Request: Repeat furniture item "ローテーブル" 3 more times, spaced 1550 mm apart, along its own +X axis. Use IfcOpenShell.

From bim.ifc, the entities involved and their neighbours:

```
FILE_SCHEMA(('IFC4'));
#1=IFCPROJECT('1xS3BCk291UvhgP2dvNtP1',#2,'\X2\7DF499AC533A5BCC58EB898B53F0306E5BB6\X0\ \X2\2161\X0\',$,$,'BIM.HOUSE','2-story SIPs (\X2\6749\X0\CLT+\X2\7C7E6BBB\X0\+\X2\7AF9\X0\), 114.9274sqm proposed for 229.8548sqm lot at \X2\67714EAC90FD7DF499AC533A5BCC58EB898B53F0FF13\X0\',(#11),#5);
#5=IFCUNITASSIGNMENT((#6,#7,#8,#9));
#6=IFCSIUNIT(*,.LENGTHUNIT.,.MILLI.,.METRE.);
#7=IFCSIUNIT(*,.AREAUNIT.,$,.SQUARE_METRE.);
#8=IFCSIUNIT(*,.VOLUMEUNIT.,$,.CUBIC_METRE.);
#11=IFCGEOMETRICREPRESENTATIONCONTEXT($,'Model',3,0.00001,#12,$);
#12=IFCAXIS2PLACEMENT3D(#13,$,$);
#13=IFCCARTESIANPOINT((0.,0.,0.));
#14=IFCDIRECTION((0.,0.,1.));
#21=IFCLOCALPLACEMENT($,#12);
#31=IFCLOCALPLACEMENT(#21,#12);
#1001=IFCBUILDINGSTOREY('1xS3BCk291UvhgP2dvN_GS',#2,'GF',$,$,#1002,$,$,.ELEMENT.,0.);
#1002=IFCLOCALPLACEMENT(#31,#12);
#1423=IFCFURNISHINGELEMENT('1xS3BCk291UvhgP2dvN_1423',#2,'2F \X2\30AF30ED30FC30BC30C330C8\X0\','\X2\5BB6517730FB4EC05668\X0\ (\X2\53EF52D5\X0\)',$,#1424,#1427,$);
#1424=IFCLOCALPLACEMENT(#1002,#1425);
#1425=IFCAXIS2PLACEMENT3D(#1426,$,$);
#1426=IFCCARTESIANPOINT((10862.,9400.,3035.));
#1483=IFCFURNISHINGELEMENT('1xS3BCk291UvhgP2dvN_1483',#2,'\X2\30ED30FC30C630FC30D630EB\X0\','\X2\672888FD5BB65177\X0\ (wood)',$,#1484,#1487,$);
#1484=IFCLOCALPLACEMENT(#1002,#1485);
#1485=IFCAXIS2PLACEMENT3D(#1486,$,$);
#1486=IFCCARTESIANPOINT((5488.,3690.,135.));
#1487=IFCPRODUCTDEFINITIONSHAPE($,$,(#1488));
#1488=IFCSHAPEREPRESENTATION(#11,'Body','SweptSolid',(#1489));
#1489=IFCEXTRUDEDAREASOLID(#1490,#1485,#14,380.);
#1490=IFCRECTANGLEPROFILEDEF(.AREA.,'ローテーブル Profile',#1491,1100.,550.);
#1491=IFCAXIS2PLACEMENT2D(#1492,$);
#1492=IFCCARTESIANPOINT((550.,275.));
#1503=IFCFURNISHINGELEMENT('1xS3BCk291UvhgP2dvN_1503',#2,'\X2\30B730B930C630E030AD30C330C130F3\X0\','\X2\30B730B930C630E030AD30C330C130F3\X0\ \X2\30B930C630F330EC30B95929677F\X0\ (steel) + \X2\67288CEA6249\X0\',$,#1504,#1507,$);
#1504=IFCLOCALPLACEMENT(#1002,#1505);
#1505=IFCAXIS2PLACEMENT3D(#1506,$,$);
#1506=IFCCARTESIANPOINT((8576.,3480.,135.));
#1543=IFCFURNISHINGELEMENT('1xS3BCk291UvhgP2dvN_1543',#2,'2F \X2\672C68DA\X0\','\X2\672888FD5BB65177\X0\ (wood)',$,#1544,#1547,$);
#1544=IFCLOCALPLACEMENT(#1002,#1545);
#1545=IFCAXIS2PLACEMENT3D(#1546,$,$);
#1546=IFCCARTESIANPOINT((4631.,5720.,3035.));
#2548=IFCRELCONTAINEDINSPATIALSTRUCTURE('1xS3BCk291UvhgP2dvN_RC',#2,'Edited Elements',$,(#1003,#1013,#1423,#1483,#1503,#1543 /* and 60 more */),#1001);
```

```python
import ifcopenshell
import ifcopenshell.api.geometry
import ifcopenshell.api.root
import ifcopenshell.util.element
import ifcopenshell.util.placement

model = ifcopenshell.open("bim.ifc")


def reuse_history(source, copy):
    """copy_class also copies each property set's owner history, people and application; keep the originals."""
    for rel in copy.IsDefinedBy:
        if rel.is_a("IfcRelDefinesByProperties") and (history := rel.RelatingPropertyDefinition.OwnerHistory):
            rel.RelatingPropertyDefinition.OwnerHistory = source.OwnerHistory
            ifcopenshell.util.element.remove_deep2(model, history)


source = model.by_guid("1xS3BCk291UvhgP2dvN_1483")
base = ifcopenshell.util.placement.get_local_placement(source.ObjectPlacement)
step = base[:3, 0] * 1550.0

for i in range(1, 4):
    copy = ifcopenshell.api.root.copy_class(model, product=source)
    copy.Representation = ifcopenshell.util.element.copy_deep(
        model, source.Representation, exclude=["IfcGeometricRepresentationContext", "IfcRepresentationMap"]
    )
    reuse_history(source, copy)
    matrix = base.copy()
    matrix[:3, 3] += i * step
    print("added at", matrix[:3, 3].round(3) + 0.0)
    ifcopenshell.api.geometry.edit_object_placement(model, product=copy, matrix=matrix, is_si=False)

model.write("bim_rev.ifc")
```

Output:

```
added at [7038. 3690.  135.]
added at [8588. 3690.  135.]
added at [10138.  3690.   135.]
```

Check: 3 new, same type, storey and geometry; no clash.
